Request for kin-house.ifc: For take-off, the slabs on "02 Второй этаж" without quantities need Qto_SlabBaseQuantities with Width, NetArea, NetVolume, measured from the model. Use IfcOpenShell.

First a look at what the model holds.

```python
import ifcopenshell
import ifcopenshell.util.element
import ifcopenshell.util.unit

model = ifcopenshell.open("kin-house.ifc")
print(model.schema)
for unit_type in ("LENGTHUNIT", "AREAUNIT", "VOLUMEUNIT"):
    print(unit_type, ifcopenshell.util.unit.calculate_unit_scale(model, unit_type))
storey = next(s for s in model.by_type("IfcBuildingStorey") if s.Name == "02 Второй этаж")
slabs = [e for e in ifcopenshell.util.element.get_decomposition(storey) if e.is_a("IfcSlab")]
for e in sorted(slabs, key=lambda e: e.id()):
    print(e.id(), e.is_a(), e.Name, list(ifcopenshell.util.element.get_psets(e, qtos_only=True)), sep=" | ")
```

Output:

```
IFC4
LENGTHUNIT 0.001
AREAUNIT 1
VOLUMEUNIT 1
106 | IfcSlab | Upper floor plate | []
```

```python
import ifcopenshell
import ifcopenshell.api.pset
import ifcopenshell.geom
import ifcopenshell.util.element
import ifcopenshell.util.shape
import ifcopenshell.util.unit

model = ifcopenshell.open("kin-house.ifc")
unit_scale = ifcopenshell.util.unit.calculate_unit_scale(model)
area_scale = ifcopenshell.util.unit.calculate_unit_scale(model, "AREAUNIT")
volume_scale = ifcopenshell.util.unit.calculate_unit_scale(model, "VOLUMEUNIT")
settings = ifcopenshell.geom.settings()

storey = next(s for s in model.by_type("IfcBuildingStorey") if s.Name == "02 Второй этаж")
slabs = [e for e in ifcopenshell.util.element.get_decomposition(storey) if e.is_a("IfcSlab")]

for e in sorted(slabs, key=lambda e: e.id()):
    if ifcopenshell.util.element.get_psets(e, qtos_only=True, should_inherit=False):
        continue
    # Geometry comes back in metres, in the element's own axes.
    shape = ifcopenshell.geom.create_shape(settings, e)
    values = {
        "Width": ifcopenshell.util.shape.get_z(shape.geometry) / unit_scale,
        "NetArea": ifcopenshell.util.shape.get_footprint_area(shape.geometry) / area_scale,
        "NetVolume": ifcopenshell.util.shape.get_volume(shape.geometry) / volume_scale,
    }
    qto = ifcopenshell.api.pset.add_qto(model, product=e, name="Qto_SlabBaseQuantities")
    ifcopenshell.api.pset.edit_qto(model, qto=qto, properties=values)
    print(e.id(), {k: round(v, 3) for k, v in values.items()})

model.write("kin-house_rev.ifc")
```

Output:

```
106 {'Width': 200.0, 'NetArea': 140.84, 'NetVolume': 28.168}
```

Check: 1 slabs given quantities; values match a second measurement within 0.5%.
